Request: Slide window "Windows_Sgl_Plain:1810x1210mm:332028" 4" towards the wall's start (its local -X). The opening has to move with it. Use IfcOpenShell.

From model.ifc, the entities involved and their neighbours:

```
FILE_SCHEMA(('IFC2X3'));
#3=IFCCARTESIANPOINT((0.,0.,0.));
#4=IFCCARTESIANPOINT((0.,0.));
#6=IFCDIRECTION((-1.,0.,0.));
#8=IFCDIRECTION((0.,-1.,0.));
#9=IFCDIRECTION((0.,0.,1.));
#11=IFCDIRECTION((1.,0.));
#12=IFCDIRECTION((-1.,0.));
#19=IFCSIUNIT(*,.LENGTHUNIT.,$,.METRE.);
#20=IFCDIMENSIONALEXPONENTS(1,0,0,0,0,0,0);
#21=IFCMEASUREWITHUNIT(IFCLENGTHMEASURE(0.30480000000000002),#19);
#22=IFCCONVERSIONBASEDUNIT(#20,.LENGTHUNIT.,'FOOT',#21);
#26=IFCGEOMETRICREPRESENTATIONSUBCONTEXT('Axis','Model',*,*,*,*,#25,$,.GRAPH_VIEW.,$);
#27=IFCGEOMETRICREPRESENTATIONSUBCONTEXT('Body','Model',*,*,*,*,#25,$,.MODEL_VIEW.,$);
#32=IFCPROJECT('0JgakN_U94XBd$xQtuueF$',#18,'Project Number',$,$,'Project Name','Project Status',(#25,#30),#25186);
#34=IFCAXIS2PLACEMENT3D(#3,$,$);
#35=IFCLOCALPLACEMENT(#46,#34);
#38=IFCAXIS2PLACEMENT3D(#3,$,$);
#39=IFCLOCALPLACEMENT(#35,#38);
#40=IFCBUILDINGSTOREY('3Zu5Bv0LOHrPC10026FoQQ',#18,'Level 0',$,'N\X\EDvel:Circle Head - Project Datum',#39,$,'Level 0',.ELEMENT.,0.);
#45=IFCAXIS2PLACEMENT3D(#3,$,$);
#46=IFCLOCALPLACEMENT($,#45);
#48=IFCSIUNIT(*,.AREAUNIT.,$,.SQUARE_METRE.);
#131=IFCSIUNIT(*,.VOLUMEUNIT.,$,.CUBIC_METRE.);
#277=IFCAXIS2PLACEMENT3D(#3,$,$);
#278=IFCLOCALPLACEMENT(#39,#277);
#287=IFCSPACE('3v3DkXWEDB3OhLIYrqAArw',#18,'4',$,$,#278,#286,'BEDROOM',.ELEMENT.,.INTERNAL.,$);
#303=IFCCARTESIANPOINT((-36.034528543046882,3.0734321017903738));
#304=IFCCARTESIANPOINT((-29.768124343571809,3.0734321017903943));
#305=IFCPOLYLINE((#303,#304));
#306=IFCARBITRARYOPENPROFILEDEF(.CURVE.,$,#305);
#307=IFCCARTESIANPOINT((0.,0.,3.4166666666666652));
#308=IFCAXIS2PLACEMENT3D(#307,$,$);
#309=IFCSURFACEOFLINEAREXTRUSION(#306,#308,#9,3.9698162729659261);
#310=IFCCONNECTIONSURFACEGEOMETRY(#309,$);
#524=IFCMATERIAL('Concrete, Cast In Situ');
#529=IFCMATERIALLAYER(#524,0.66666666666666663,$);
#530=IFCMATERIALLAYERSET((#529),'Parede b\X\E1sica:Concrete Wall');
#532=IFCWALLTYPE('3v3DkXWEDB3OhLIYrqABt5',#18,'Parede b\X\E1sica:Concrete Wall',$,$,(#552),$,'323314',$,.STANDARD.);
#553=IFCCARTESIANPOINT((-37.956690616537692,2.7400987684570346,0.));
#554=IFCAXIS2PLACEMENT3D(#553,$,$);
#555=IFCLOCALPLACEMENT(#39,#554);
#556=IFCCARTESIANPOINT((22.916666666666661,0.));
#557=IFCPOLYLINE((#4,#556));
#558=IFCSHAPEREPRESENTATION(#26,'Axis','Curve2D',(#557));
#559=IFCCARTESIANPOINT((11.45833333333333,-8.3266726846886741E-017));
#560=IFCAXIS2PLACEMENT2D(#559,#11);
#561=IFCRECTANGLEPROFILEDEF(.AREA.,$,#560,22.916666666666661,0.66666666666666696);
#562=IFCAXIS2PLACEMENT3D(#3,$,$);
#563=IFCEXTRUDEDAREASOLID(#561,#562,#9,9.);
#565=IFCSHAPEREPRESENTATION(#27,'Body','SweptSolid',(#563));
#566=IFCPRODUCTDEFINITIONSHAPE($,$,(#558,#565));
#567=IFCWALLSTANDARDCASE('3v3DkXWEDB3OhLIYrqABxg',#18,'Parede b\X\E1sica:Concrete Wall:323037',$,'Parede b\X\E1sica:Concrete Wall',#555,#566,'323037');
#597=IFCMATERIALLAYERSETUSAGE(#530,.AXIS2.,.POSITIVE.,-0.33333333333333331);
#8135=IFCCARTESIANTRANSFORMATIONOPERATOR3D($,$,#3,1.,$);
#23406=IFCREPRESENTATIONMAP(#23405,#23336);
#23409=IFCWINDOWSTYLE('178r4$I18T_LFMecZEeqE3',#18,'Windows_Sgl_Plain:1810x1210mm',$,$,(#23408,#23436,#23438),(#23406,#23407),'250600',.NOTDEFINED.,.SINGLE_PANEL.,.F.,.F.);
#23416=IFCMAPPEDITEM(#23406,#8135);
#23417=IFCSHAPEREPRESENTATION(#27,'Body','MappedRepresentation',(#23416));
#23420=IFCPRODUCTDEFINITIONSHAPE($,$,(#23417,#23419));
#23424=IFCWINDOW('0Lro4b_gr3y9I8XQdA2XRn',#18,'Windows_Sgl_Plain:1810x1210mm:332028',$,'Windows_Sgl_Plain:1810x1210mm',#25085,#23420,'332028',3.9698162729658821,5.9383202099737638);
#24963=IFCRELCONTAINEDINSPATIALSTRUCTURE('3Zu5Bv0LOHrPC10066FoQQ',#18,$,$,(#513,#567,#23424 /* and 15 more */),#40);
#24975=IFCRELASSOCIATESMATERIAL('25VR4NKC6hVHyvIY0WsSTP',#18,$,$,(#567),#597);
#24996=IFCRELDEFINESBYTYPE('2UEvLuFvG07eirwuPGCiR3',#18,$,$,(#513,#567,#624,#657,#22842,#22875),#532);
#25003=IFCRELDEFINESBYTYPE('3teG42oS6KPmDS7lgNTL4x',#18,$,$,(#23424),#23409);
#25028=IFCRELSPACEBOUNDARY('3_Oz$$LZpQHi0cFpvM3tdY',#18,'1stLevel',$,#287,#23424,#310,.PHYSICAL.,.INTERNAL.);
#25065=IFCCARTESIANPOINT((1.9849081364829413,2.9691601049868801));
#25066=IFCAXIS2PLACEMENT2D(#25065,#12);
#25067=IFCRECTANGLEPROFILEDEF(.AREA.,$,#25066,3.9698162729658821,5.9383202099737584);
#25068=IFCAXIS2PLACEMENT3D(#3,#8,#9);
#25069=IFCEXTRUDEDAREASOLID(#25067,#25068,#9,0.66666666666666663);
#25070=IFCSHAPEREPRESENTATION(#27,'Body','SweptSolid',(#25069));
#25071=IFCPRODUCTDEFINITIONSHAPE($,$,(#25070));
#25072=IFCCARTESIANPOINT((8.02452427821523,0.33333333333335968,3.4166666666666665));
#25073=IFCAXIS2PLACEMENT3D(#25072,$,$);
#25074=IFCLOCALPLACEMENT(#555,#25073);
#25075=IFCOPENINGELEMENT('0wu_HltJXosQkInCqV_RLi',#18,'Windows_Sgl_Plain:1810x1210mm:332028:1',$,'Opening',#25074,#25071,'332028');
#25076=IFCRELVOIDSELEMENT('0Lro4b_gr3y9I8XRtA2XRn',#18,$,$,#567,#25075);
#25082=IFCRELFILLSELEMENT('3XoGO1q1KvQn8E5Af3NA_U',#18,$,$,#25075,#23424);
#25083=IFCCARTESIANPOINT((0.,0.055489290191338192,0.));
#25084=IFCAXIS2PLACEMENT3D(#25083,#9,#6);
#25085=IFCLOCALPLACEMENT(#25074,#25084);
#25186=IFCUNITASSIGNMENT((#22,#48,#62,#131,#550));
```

```python
import numpy as np
import ifcopenshell
import ifcopenshell.api.geometry
import ifcopenshell.util.placement
import ifcopenshell.util.unit

model = ifcopenshell.open("model.ifc")
unit_scale = ifcopenshell.util.unit.calculate_unit_scale(model)

window = model.by_guid("0Lro4b_gr3y9I8XQdA2XRn")
opening = window.FillsVoids[0].RelatingOpeningElement
wall = opening.VoidsElements[0].RelatingBuildingElement

wall_matrix = ifcopenshell.util.placement.get_local_placement(wall.ObjectPlacement)
shift = wall_matrix[:3, 0] * -4 * 0.0254 / unit_scale
before = ifcopenshell.util.placement.get_local_placement(window.ObjectPlacement)[:3, 3].copy()

# The window is placed relative to its opening, so it follows when the opening moves.
matrix = ifcopenshell.util.placement.get_local_placement(opening.ObjectPlacement)
matrix[:3, 3] += shift
ifcopenshell.api.geometry.edit_object_placement(
    model, product=opening, matrix=matrix, is_si=False, should_transform_children=True
)

# Space boundary surfaces are stored in each space's coordinates; move them too.
for rel in window.ProvidesBoundaries:
    if not rel.ConnectionGeometry:
        continue
    surface = rel.ConnectionGeometry.SurfaceOnRelatingElement
    space_matrix = ifcopenshell.util.placement.get_local_placement(rel.RelatingSpace.ObjectPlacement)
    point = np.array(surface.Position.Location.Coordinates) + space_matrix[:3, :3].T @ shift
    surface.Position = model.createIfcAxis2Placement3D(
        model.createIfcCartesianPoint(point.tolist()), surface.Position.Axis, surface.Position.RefDirection
    )

after = ifcopenshell.util.placement.get_local_placement(window.ObjectPlacement)[:3, 3]
print("window moved by", (after - before).round(3) + 0.0)

model.write("model_edited.ifc")
```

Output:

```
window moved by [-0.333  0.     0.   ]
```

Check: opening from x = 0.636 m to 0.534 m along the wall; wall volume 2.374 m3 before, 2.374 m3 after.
